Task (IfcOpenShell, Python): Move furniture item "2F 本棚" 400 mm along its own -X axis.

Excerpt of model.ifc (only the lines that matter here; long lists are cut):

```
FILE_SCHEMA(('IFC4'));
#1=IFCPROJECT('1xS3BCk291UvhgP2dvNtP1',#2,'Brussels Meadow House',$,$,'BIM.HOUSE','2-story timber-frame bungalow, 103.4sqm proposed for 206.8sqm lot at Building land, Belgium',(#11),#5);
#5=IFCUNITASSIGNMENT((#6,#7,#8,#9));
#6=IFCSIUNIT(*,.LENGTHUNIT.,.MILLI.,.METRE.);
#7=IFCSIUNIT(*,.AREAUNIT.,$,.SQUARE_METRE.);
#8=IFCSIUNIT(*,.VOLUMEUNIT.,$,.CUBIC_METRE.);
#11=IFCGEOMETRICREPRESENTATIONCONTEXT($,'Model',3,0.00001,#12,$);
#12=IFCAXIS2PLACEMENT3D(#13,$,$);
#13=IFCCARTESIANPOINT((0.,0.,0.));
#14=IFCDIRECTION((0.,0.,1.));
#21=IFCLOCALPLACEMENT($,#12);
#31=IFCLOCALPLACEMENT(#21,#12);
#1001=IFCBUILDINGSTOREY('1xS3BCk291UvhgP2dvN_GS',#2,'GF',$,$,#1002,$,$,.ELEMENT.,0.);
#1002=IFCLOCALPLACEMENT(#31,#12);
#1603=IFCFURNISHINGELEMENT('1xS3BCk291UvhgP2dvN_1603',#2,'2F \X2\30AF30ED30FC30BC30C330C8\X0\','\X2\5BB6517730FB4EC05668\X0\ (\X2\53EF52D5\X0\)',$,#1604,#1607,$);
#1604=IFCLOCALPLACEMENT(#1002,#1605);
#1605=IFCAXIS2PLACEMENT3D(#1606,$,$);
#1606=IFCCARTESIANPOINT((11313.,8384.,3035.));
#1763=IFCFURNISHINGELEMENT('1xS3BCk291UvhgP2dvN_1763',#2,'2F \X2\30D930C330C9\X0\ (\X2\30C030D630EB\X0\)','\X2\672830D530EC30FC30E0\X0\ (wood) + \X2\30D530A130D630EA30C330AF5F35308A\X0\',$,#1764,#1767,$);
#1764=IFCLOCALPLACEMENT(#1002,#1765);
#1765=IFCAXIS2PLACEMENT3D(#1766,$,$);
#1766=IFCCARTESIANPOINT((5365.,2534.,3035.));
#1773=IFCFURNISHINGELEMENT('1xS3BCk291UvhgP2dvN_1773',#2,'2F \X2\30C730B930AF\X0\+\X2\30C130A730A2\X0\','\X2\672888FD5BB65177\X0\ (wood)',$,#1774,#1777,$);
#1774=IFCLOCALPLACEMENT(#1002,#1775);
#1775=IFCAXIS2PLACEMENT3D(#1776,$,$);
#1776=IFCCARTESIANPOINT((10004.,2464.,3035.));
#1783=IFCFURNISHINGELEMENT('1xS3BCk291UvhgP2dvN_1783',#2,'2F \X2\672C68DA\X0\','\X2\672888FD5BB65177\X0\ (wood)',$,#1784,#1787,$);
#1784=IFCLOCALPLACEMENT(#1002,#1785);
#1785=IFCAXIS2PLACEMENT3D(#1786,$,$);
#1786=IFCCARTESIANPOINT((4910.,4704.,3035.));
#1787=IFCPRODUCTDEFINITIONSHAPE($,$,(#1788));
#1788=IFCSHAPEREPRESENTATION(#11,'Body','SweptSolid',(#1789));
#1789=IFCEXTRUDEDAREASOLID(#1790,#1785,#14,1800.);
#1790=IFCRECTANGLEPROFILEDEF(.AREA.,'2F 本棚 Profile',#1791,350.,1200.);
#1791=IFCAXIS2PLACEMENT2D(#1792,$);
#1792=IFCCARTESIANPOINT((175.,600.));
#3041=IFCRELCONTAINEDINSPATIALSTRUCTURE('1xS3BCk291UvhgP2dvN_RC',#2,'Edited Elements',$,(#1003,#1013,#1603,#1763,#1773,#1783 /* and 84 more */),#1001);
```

```python
import ifcopenshell
import ifcopenshell.api.geometry
import ifcopenshell.util.placement
import ifcopenshell.util.unit

model = ifcopenshell.open("model.ifc")
unit_scale = ifcopenshell.util.unit.calculate_unit_scale(model)

item = model.by_guid("1xS3BCk291UvhgP2dvN_1783")
matrix = ifcopenshell.util.placement.get_local_placement(item.ObjectPlacement)
matrix[:3, 3] -= matrix[:3, 0] * 0.4 / unit_scale
ifcopenshell.api.geometry.edit_object_placement(model, product=item, matrix=matrix, is_si=False)

print(ifcopenshell.util.placement.get_local_placement(item.ObjectPlacement).round(3) + 0.0)

model.write("model_v2.ifc")
```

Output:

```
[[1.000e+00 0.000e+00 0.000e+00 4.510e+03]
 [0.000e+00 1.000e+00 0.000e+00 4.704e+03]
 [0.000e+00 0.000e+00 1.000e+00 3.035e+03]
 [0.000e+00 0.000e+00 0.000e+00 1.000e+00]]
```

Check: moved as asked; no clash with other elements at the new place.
